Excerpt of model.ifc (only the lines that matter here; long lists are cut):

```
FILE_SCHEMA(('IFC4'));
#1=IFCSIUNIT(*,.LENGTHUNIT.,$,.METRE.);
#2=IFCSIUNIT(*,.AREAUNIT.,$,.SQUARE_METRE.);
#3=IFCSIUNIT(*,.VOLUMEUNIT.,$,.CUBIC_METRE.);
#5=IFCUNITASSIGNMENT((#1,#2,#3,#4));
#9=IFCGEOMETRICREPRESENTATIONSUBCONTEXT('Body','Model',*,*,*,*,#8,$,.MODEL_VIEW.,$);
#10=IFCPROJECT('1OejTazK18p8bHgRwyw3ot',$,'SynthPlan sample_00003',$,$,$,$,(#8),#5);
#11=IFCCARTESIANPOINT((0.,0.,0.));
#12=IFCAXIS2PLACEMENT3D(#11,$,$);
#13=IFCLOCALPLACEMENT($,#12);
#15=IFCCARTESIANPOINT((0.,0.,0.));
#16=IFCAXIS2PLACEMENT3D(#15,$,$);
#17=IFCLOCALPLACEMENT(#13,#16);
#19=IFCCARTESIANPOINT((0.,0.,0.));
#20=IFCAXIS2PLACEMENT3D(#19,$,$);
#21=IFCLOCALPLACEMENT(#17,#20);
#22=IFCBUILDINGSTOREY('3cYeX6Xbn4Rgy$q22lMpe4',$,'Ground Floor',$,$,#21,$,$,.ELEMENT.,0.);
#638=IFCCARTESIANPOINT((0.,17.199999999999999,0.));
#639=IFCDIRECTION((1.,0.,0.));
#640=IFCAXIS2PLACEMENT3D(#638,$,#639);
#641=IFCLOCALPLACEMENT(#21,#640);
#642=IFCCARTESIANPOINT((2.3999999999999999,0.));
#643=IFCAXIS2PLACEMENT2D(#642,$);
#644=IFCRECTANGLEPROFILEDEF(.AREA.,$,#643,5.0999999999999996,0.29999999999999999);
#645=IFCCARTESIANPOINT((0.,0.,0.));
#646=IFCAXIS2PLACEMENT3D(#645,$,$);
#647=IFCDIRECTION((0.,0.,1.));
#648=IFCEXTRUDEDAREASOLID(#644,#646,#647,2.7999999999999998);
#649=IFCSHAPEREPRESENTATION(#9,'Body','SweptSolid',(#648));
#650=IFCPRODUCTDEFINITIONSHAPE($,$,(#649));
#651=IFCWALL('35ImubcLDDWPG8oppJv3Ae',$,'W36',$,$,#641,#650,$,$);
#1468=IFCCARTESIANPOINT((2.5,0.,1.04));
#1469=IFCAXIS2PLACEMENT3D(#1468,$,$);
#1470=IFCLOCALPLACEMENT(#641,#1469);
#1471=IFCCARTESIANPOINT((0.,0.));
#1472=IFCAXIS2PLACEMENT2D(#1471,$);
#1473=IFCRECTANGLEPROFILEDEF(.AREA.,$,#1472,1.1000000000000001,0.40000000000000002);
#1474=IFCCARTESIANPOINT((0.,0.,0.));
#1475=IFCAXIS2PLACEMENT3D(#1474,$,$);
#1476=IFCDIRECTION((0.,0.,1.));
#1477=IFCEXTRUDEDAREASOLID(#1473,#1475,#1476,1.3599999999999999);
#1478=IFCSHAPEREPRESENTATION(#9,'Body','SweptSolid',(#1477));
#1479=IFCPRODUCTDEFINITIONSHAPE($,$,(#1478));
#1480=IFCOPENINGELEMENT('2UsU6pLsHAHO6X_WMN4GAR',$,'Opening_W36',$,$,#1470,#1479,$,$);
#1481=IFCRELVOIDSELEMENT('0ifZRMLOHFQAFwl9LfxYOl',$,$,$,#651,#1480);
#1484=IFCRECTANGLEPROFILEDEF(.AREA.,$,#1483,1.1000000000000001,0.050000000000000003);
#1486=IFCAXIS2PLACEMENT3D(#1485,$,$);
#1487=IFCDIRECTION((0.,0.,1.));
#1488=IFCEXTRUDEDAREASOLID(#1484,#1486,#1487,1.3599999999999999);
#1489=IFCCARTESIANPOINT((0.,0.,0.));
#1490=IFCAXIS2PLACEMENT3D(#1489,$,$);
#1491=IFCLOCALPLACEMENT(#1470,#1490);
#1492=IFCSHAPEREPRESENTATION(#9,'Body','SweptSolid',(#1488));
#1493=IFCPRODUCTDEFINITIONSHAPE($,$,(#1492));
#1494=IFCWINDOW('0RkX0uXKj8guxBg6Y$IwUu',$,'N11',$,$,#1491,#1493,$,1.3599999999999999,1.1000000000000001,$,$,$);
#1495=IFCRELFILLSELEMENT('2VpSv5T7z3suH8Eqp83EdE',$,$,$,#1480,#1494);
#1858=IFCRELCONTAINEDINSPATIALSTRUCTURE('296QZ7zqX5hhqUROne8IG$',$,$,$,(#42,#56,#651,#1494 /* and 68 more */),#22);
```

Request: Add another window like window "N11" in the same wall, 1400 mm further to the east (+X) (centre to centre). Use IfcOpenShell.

```python
import ifcopenshell
import ifcopenshell.api.feature
import ifcopenshell.api.geometry
import ifcopenshell.api.root
import ifcopenshell.geom
import ifcopenshell.util.element
import ifcopenshell.util.placement
import ifcopenshell.util.shape
import ifcopenshell.util.unit

model = ifcopenshell.open("model.ifc")
unit_scale = ifcopenshell.util.unit.calculate_unit_scale(model)
settings = ifcopenshell.geom.settings()


def volume(element):
    """Net volume in cubic metres, openings subtracted."""
    shape = ifcopenshell.geom.create_shape(settings, element)
    return ifcopenshell.util.shape.get_volume(shape.geometry)


window = model.by_id(1494)
opening = window.FillsVoids[0].RelatingOpeningElement
wall = opening.VoidsElements[0].RelatingBuildingElement
before = volume(wall)
shift = ifcopenshell.util.placement.get_local_placement(wall.ObjectPlacement)[:3, 0] * 1.4 / unit_scale

# copy_class copies the void relationship, type, container and properties, but no geometry.
new_opening = ifcopenshell.api.root.copy_class(model, product=opening)
new_opening.Representation = ifcopenshell.util.element.copy_deep(
    model, opening.Representation, exclude=["IfcGeometricRepresentationContext", "IfcRepresentationMap"]
)
new_window = ifcopenshell.api.root.copy_class(model, product=window)
new_window.Representation = ifcopenshell.util.element.copy_deep(
    model, window.Representation, exclude=["IfcGeometricRepresentationContext", "IfcRepresentationMap"]
)
ifcopenshell.api.feature.add_filling(model, opening=new_opening, element=new_window)

for old, new in ((opening, new_opening), (window, new_window)):
    matrix = ifcopenshell.util.placement.get_local_placement(old.ObjectPlacement)
    matrix[:3, 3] += shift
    ifcopenshell.api.geometry.edit_object_placement(model, product=new, matrix=matrix, is_si=False)

after = volume(wall)

print(f"wall volume {before:.3f} -> {after:.3f} m3")

model.write("model_edited.ifc")
```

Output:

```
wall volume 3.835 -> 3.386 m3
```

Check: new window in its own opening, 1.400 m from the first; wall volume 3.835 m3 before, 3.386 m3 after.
